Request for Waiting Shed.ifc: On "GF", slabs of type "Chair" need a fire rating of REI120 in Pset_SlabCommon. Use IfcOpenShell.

First a look at what the model holds.

```python
import ifcopenshell
import ifcopenshell.util.element

model = ifcopenshell.open("Waiting Shed.ifc")
print(model.schema)
storey = next(s for s in model.by_type("IfcBuildingStorey") if s.Name == "GF")
slabs = [e for e in ifcopenshell.util.element.get_decomposition(storey) if e.is_a("IfcSlab")]
seen = {}
for e in slabs:
    element_type = ifcopenshell.util.element.get_type(e)
    key = (element_type.Name if element_type != e and element_type else None, ifcopenshell.util.element.get_pset(e, "Pset_SlabCommon", "FireRating"))
    seen[key] = seen.get(key, 0) + 1
for (name, value), count in sorted(seen.items(), key=str):
    print(count, "x", name, "|", value)
```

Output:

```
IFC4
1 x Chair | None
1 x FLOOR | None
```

```python
import ifcopenshell
import ifcopenshell.api.pset
import ifcopenshell.util.element

model = ifcopenshell.open("Waiting Shed.ifc")

storey = next(s for s in model.by_type("IfcBuildingStorey") if s.Name == "GF")
slabs = [e for e in ifcopenshell.util.element.get_decomposition(storey) if e.is_a("IfcSlab")]

count = 0
for e in slabs:
    element_type = ifcopenshell.util.element.get_type(e)
    if element_type in (None, e) or element_type.Name != "Chair":
        continue
    # add_pset returns the element's existing set when there is one.
    pset = ifcopenshell.api.pset.add_pset(model, product=e, name="Pset_SlabCommon")
    ifcopenshell.api.pset.edit_pset(model, pset=pset, properties={"FireRating": "REI120"})
    count += 1

print(count, "slabs updated")

model.write("Waiting Shed_v2.ifc")
```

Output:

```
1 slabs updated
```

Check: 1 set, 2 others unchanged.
